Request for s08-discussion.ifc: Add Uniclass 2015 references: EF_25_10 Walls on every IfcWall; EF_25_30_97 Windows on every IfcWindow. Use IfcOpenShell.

First a look at what the model holds.

```python
import ifcopenshell

model = ifcopenshell.open("s08-discussion.ifc")
print(model.schema)
print("classifications:", [c.Name for c in model.by_type("IfcClassification")])
for ifc_class in ("IfcDoor", "IfcRoof", "IfcStair", "IfcWall", "IfcWindow"):
    print(ifc_class, len(model.by_type(ifc_class)))
```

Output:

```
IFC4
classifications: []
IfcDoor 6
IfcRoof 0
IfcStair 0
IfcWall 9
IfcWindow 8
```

```python
import ifcopenshell
import ifcopenshell.api.classification

model = ifcopenshell.open("s08-discussion.ifc")

system = ifcopenshell.api.classification.add_classification(model, classification="Uniclass 2015")

codes = {
    "IfcWall": ("EF_25_10", "Walls"),
    "IfcWindow": ("EF_25_30_97", "Windows"),
}
for ifc_class, (code, name) in codes.items():
    products = model.by_type(ifc_class)
    ifcopenshell.api.classification.add_reference(
        model, products=products, classification=system, identification=code, name=name
    )
    print(code, len(products))

model.write("s08-discussion_v2.ifc")
```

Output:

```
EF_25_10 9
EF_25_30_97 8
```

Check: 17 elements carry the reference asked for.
